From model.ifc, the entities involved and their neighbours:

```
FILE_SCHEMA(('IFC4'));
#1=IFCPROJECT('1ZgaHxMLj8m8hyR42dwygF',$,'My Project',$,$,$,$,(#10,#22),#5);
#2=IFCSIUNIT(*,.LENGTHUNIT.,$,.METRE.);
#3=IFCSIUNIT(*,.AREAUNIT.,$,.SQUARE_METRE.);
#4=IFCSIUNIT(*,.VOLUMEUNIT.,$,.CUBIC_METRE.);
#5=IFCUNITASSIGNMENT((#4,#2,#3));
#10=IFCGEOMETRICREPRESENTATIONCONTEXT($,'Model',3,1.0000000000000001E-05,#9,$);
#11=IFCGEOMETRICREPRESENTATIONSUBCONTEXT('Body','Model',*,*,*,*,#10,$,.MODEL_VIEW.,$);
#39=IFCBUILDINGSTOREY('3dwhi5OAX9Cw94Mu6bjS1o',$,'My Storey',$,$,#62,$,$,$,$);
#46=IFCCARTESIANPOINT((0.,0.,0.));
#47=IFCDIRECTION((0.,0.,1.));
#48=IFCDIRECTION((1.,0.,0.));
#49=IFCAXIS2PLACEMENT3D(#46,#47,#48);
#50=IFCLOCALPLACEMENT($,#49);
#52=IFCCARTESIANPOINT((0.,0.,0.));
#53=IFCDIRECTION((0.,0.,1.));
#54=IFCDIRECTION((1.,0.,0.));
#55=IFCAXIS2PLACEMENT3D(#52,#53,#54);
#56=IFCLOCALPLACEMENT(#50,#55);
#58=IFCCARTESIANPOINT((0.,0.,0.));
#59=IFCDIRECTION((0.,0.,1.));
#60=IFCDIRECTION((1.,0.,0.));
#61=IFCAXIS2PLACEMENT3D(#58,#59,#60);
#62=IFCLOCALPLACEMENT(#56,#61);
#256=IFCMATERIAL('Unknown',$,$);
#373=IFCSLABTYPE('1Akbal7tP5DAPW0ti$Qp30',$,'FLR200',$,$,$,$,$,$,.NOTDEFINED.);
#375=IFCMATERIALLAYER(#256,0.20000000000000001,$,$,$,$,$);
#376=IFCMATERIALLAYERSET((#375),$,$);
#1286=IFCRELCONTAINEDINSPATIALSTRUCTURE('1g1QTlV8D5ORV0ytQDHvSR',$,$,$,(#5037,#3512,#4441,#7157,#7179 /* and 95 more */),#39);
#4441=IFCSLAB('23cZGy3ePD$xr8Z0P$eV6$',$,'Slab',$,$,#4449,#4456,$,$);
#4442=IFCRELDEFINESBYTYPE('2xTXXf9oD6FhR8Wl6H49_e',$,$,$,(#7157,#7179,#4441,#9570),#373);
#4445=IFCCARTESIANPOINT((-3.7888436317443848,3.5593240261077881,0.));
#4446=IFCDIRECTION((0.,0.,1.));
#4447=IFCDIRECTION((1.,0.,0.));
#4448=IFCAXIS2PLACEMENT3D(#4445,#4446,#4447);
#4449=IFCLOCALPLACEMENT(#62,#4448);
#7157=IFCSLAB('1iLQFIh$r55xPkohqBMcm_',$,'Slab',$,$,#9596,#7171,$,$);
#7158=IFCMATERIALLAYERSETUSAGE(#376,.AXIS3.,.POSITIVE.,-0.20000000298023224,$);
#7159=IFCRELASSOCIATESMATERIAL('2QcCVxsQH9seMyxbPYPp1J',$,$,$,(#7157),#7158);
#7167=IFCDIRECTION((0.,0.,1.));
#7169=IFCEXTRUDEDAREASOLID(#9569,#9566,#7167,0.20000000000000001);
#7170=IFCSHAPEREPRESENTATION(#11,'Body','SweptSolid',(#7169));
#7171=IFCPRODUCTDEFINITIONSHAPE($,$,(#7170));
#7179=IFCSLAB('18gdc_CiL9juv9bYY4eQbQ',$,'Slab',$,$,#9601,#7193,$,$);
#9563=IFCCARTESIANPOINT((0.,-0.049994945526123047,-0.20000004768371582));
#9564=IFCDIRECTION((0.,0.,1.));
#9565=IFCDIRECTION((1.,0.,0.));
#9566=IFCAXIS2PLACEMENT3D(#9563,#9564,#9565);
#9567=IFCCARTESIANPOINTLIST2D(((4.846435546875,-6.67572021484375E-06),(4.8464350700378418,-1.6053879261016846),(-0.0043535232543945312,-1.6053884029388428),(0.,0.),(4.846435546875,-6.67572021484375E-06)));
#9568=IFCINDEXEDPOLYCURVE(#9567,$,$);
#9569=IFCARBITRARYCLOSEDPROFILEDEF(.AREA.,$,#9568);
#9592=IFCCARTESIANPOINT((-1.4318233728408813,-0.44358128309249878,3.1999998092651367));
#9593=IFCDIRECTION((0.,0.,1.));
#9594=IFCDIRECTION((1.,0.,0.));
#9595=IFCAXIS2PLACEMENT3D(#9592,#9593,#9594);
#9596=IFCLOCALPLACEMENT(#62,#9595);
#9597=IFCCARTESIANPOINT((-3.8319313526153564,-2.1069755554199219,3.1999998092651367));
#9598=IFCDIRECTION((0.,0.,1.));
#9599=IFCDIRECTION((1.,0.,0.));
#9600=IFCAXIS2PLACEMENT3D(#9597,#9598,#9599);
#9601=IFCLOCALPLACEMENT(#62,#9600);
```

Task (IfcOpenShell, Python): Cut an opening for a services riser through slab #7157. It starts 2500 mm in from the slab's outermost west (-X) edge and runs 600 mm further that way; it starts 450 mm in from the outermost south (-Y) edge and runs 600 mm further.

```python
import numpy as np
import ifcopenshell
import ifcopenshell.api.feature
import ifcopenshell.api.geometry
import ifcopenshell.api.root
import ifcopenshell.geom
import ifcopenshell.util.placement
import ifcopenshell.util.representation
import ifcopenshell.util.shape
import ifcopenshell.util.unit

model = ifcopenshell.open("model.ifc")
unit_scale = ifcopenshell.util.unit.calculate_unit_scale(model)
settings = ifcopenshell.geom.settings()


def volume(element):
    """Net volume in cubic metres, openings subtracted."""
    shape = ifcopenshell.geom.create_shape(settings, element)
    return ifcopenshell.util.shape.get_volume(shape.geometry)


slab = model.by_id(7157)
before = volume(slab)

# Extent in the slab's own axes, in metres. The edges named are its -X and -Y sides.
slab_shape = ifcopenshell.geom.create_shape(settings, slab)
vertices = ifcopenshell.util.shape.get_vertices(slab_shape.geometry)
x_min, y_min, bottom = vertices.min(axis=0)
top = vertices[:, 2].max()

opening = ifcopenshell.api.root.create_entity(model, ifc_class="IfcOpeningElement", name="Services riser opening", predefined_type="OPENING")
context = ifcopenshell.util.representation.get_context(model, "Model", "Body", "MODEL_VIEW")
width, depth = 0.6, 0.6
outline = [(0.0, 0.0), (width, 0.0), (width, depth), (0.0, depth), (0.0, 0.0)]
# Overshoot both faces by 50 mm so the cut is clean.
shape = ifcopenshell.api.geometry.add_slab_representation(
    model, context=context, depth=top - bottom + 0.1, polyline=outline
)
ifcopenshell.api.geometry.assign_representation(model, product=opening, representation=shape)

matrix = ifcopenshell.util.placement.get_local_placement(slab.ObjectPlacement)
matrix[:, 3] = matrix @ np.append(np.array([x_min + 2.5, y_min + 0.45, bottom - 0.05]) / unit_scale, 1.0)
ifcopenshell.api.geometry.edit_object_placement(model, product=opening, matrix=matrix, is_si=False)
ifcopenshell.api.feature.add_feature(model, feature=opening, element=slab)

after = volume(slab)

print(f"slab volume {before:.3f} -> {after:.3f} m3")

model.write("model-out.ifc")
```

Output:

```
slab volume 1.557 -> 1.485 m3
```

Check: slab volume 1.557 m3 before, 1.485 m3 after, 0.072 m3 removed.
